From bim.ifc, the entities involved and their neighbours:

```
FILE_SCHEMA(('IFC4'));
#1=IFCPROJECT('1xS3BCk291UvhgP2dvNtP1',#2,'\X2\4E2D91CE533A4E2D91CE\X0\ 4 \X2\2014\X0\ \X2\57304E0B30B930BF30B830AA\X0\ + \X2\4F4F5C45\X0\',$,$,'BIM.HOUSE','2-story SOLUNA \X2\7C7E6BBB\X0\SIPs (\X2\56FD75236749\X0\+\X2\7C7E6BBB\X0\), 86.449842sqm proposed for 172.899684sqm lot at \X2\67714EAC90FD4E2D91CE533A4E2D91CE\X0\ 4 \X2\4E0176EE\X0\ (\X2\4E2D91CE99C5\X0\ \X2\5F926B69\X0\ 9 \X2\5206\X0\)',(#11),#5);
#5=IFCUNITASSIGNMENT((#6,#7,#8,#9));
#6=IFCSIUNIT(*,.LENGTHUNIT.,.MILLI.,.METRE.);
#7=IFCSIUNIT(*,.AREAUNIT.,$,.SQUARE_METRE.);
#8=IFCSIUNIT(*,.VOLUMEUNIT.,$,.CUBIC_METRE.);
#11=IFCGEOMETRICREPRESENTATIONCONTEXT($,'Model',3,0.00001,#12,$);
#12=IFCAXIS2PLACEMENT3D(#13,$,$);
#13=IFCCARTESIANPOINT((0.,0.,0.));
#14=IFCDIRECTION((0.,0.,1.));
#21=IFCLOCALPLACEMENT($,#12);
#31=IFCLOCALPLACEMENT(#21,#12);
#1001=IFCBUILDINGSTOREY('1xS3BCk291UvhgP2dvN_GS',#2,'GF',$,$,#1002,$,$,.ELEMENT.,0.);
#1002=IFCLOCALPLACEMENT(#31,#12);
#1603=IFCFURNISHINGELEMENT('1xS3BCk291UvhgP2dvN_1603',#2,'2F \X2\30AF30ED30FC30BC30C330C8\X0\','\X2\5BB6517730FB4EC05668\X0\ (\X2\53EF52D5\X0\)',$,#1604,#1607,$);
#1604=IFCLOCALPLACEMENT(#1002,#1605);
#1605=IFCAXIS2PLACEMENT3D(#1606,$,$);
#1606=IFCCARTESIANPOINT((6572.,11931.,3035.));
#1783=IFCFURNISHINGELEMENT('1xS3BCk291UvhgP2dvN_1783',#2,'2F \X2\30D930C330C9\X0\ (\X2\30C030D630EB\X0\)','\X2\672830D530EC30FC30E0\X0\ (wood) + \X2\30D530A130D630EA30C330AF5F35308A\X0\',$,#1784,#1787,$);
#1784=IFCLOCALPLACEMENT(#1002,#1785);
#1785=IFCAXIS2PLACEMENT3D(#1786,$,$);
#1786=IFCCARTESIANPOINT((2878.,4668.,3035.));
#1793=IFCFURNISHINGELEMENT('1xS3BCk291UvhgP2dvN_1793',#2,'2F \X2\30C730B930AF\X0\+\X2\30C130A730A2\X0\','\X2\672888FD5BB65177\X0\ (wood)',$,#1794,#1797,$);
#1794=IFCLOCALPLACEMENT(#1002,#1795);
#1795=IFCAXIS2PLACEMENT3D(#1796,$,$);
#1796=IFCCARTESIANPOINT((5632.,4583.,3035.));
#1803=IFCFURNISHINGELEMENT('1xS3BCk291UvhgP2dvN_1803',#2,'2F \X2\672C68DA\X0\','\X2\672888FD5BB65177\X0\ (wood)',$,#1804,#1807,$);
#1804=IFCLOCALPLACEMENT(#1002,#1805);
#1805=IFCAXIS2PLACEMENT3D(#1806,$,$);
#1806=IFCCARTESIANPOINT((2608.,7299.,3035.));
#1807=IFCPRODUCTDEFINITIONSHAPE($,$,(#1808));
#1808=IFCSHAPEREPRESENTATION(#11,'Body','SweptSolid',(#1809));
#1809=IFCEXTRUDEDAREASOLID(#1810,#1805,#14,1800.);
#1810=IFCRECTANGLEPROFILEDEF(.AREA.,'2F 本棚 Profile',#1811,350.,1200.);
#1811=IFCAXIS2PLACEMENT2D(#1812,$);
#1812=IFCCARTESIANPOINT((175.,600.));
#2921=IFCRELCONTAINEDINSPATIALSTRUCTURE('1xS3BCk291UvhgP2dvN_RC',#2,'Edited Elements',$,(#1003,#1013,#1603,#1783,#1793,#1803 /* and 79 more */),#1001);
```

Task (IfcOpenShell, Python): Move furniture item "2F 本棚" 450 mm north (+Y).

```python
import ifcopenshell
import ifcopenshell.api.geometry
import ifcopenshell.util.placement

model = ifcopenshell.open("bim.ifc")

item = model.by_guid("1xS3BCk291UvhgP2dvN_1803")
matrix = ifcopenshell.util.placement.get_local_placement(item.ObjectPlacement)
matrix[1, 3] += 450.0
ifcopenshell.api.geometry.edit_object_placement(model, product=item, matrix=matrix, is_si=False)

print(ifcopenshell.util.placement.get_local_placement(item.ObjectPlacement).round(3) + 0.0)

model.write("bim_edited.ifc")
```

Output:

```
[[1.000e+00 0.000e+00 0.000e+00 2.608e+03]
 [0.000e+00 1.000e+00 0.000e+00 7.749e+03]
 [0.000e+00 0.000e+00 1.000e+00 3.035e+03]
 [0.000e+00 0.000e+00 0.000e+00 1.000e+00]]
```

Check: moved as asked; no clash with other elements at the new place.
